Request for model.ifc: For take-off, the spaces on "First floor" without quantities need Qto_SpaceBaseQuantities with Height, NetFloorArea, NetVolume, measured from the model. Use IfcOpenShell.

First a look at what the model holds.

```python
import ifcopenshell
import ifcopenshell.util.element
import ifcopenshell.util.unit

model = ifcopenshell.open("model.ifc")
print(model.schema)
for unit_type in ("LENGTHUNIT", "AREAUNIT", "VOLUMEUNIT"):
    print(unit_type, ifcopenshell.util.unit.calculate_unit_scale(model, unit_type))
storey = next(s for s in model.by_type("IfcBuildingStorey") if s.Name == "First floor")
spaces = [e for e in ifcopenshell.util.element.get_decomposition(storey) if e.is_a("IfcSpace")]
for e in sorted(spaces, key=lambda e: e.id()):
    print(e.id(), e.is_a(), e.Name, list(ifcopenshell.util.element.get_psets(e, qtos_only=True)), sep=" | ")
```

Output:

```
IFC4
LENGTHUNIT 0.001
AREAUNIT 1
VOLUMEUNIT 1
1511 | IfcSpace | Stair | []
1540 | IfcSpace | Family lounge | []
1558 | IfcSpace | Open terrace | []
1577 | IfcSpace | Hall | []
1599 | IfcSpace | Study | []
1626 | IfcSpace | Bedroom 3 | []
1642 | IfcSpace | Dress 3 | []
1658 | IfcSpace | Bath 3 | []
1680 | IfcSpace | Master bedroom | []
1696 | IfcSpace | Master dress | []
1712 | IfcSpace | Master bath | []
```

```python
import ifcopenshell
import ifcopenshell.api.pset
import ifcopenshell.geom
import ifcopenshell.util.element
import ifcopenshell.util.shape
import ifcopenshell.util.unit

model = ifcopenshell.open("model.ifc")
unit_scale = ifcopenshell.util.unit.calculate_unit_scale(model)
area_scale = ifcopenshell.util.unit.calculate_unit_scale(model, "AREAUNIT")
volume_scale = ifcopenshell.util.unit.calculate_unit_scale(model, "VOLUMEUNIT")
settings = ifcopenshell.geom.settings()

storey = next(s for s in model.by_type("IfcBuildingStorey") if s.Name == "First floor")
spaces = [e for e in ifcopenshell.util.element.get_decomposition(storey) if e.is_a("IfcSpace")]

for e in sorted(spaces, key=lambda e: e.id()):
    if ifcopenshell.util.element.get_psets(e, qtos_only=True, should_inherit=False):
        continue
    # Geometry comes back in metres, in the element's own axes.
    shape = ifcopenshell.geom.create_shape(settings, e)
    values = {
        "Height": ifcopenshell.util.shape.get_z(shape.geometry) / unit_scale,
        "NetFloorArea": ifcopenshell.util.shape.get_footprint_area(shape.geometry) / area_scale,
        "NetVolume": ifcopenshell.util.shape.get_volume(shape.geometry) / volume_scale,
    }
    qto = ifcopenshell.api.pset.add_qto(model, product=e, name="Qto_SpaceBaseQuantities")
    ifcopenshell.api.pset.edit_qto(model, qto=qto, properties=values)
    print(e.id(), {k: round(v, 3) for k, v in values.items()})

model.write("model_edited.ifc")
```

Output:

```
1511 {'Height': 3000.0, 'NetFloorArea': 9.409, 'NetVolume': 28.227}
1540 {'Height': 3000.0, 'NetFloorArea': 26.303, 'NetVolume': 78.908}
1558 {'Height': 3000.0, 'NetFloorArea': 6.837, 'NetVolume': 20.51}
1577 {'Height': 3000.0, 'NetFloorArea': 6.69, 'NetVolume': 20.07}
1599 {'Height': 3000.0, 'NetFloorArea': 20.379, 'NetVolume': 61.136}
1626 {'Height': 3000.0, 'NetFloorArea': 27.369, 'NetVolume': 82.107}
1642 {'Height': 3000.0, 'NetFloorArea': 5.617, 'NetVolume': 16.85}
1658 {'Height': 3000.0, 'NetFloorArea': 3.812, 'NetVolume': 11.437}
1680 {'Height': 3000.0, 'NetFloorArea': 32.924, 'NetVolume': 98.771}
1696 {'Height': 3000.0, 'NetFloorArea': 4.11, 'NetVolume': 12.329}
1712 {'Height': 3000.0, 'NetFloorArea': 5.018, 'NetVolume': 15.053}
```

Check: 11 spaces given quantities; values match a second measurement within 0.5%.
